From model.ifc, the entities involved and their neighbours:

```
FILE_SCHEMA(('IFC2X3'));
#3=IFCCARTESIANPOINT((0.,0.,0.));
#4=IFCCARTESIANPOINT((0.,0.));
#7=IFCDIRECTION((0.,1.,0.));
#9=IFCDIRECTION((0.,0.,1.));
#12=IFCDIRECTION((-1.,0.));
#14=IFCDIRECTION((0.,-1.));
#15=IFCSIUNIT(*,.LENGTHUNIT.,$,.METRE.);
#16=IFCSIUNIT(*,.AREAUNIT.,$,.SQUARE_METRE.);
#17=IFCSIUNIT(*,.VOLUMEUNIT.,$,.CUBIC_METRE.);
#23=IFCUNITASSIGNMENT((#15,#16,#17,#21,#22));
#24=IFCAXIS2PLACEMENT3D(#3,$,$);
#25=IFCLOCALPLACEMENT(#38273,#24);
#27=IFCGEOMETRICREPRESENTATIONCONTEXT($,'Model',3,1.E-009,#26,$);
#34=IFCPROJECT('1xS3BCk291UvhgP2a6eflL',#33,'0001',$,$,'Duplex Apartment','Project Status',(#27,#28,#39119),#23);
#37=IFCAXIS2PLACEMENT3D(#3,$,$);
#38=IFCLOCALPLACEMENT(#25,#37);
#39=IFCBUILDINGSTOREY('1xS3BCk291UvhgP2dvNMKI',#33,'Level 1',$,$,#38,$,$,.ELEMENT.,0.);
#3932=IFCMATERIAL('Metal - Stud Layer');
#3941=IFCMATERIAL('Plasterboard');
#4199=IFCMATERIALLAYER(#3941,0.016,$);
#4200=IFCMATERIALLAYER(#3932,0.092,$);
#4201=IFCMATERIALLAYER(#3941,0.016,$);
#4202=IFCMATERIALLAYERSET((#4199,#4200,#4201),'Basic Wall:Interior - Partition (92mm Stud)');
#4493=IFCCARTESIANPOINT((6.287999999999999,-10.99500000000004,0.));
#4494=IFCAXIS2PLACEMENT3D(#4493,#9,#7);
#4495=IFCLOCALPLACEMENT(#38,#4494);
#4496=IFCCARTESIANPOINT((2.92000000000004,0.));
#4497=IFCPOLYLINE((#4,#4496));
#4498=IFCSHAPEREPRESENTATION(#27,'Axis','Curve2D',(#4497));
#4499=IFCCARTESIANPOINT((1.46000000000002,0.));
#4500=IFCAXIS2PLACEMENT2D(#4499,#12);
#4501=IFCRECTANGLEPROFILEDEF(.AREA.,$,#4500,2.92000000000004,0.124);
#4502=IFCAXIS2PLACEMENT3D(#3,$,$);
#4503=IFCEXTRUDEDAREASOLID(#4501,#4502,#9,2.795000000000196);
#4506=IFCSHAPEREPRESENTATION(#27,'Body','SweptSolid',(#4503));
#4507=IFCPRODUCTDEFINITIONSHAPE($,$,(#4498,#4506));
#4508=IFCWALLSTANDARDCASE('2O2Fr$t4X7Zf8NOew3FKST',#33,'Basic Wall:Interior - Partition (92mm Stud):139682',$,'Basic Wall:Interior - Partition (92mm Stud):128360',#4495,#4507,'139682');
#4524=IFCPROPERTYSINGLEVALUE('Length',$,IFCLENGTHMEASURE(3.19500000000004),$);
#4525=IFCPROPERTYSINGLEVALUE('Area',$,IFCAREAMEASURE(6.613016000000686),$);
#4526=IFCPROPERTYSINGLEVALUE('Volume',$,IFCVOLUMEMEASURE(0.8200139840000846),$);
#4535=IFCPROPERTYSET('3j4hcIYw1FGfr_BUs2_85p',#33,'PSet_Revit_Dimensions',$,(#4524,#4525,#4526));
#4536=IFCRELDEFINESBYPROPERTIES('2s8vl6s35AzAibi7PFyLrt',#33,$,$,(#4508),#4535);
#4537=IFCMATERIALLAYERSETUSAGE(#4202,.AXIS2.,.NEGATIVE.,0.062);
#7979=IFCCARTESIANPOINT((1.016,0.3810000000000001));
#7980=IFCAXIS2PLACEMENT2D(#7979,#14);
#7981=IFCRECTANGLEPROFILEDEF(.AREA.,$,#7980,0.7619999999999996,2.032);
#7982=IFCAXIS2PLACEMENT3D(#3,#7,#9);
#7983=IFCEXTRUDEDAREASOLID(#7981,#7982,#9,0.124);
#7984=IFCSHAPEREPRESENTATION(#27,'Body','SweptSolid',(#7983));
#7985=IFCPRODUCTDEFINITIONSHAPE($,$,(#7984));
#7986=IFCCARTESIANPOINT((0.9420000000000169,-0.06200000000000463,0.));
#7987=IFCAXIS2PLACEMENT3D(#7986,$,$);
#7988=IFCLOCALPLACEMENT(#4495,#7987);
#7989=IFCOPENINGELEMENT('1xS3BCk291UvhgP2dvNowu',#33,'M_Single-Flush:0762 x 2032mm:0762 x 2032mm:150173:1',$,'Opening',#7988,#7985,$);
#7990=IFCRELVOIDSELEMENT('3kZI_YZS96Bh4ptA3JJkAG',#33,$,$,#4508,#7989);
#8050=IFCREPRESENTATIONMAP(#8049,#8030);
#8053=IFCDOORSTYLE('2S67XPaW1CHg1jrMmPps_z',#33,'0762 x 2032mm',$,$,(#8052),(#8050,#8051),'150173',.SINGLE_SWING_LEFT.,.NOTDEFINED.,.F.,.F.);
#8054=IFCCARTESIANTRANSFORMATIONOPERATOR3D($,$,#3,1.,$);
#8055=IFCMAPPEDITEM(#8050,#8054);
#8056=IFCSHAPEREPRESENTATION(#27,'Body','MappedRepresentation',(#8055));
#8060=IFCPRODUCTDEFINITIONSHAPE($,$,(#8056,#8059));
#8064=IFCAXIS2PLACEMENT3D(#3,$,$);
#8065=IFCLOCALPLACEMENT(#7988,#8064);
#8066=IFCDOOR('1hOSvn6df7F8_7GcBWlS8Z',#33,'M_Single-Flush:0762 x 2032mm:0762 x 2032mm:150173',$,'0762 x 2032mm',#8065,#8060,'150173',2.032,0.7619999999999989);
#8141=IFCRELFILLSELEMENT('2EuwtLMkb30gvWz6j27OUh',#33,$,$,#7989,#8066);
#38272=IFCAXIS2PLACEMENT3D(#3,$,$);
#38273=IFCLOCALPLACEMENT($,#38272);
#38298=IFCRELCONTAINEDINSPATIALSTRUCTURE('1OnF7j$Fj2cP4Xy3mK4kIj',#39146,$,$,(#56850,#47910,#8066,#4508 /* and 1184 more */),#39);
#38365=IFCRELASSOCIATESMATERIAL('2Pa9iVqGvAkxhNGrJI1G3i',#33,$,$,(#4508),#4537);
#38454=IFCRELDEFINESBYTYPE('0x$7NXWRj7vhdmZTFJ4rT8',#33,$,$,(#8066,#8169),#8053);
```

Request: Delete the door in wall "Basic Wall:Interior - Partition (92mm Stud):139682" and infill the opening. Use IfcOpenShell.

```python
import ifcopenshell
import ifcopenshell.api.feature
import ifcopenshell.api.pset
import ifcopenshell.api.root
import ifcopenshell.geom
import ifcopenshell.util.element
import ifcopenshell.util.shape
import ifcopenshell.util.unit

model = ifcopenshell.open("model.ifc")
area_scale = ifcopenshell.util.unit.calculate_unit_scale(model, "AREAUNIT")
volume_scale = ifcopenshell.util.unit.calculate_unit_scale(model, "VOLUMEUNIT")
settings = ifcopenshell.geom.settings()


def volume(element):
    """Net volume in cubic metres, openings subtracted."""
    shape = ifcopenshell.geom.create_shape(settings, element)
    return ifcopenshell.util.shape.get_volume(shape.geometry)


door = model.by_guid("1hOSvn6df7F8_7GcBWlS8Z")
opening = door.FillsVoids[0].RelatingOpeningElement
wall = opening.VoidsElements[0].RelatingBuildingElement
before = volume(wall)

ifcopenshell.api.root.remove_product(model, product=door)
ifcopenshell.api.feature.remove_feature(model, feature=opening)

after = volume(wall)
thickness = 0.124  # wall thickness in metres

# Update the wall's stored quantities.
pset = model.by_id(ifcopenshell.util.element.get_pset(wall, "PSet_Revit_Dimensions", should_inherit=False)["id"])
ifcopenshell.api.pset.edit_pset(model, pset=pset, properties={
    "Area": model.create_entity("IfcAreaMeasure", after / thickness / area_scale),
    "Volume": model.create_entity("IfcVolumeMeasure", after / volume_scale),
})

print(f"wall volume {before:.3f} -> {after:.3f} m3")

model.write("model_edited.ifc")
```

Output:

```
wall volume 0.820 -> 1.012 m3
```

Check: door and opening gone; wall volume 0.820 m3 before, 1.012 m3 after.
